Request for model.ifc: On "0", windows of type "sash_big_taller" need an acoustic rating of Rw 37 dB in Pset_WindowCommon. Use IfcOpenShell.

First a look at what the model holds.

```python
import ifcopenshell
import ifcopenshell.util.element

model = ifcopenshell.open("model.ifc")
print(model.schema)
storey = next(s for s in model.by_type("IfcBuildingStorey") if s.Name == "0")
windows = [e for e in ifcopenshell.util.element.get_decomposition(storey) if e.is_a("IfcWindow")]
seen = {}
for e in windows:
    element_type = ifcopenshell.util.element.get_type(e)
    key = (element_type.Name if element_type != e and element_type else None, ifcopenshell.util.element.get_pset(e, "Pset_WindowCommon", "AcousticRating"))
    seen[key] = seen.get(key, 0) + 1
for (name, value), count in sorted(seen.items(), key=str):
    print(count, "x", name, "|", value)
```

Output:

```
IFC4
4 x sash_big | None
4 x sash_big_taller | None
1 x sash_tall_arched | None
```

```python
import ifcopenshell
import ifcopenshell.api.pset
import ifcopenshell.util.element

model = ifcopenshell.open("model.ifc")

storey = next(s for s in model.by_type("IfcBuildingStorey") if s.Name == "0")
windows = [e for e in ifcopenshell.util.element.get_decomposition(storey) if e.is_a("IfcWindow")]

count = 0
for e in windows:
    element_type = ifcopenshell.util.element.get_type(e)
    if element_type in (None, e) or element_type.Name != "sash_big_taller":
        continue
    # add_pset returns the element's existing set when there is one.
    pset = ifcopenshell.api.pset.add_pset(model, product=e, name="Pset_WindowCommon")
    ifcopenshell.api.pset.edit_pset(model, pset=pset, properties={"AcousticRating": "Rw 37 dB"})
    count += 1

print(count, "windows updated")

model.write("model_rev.ifc")
```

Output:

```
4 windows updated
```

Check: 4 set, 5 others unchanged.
